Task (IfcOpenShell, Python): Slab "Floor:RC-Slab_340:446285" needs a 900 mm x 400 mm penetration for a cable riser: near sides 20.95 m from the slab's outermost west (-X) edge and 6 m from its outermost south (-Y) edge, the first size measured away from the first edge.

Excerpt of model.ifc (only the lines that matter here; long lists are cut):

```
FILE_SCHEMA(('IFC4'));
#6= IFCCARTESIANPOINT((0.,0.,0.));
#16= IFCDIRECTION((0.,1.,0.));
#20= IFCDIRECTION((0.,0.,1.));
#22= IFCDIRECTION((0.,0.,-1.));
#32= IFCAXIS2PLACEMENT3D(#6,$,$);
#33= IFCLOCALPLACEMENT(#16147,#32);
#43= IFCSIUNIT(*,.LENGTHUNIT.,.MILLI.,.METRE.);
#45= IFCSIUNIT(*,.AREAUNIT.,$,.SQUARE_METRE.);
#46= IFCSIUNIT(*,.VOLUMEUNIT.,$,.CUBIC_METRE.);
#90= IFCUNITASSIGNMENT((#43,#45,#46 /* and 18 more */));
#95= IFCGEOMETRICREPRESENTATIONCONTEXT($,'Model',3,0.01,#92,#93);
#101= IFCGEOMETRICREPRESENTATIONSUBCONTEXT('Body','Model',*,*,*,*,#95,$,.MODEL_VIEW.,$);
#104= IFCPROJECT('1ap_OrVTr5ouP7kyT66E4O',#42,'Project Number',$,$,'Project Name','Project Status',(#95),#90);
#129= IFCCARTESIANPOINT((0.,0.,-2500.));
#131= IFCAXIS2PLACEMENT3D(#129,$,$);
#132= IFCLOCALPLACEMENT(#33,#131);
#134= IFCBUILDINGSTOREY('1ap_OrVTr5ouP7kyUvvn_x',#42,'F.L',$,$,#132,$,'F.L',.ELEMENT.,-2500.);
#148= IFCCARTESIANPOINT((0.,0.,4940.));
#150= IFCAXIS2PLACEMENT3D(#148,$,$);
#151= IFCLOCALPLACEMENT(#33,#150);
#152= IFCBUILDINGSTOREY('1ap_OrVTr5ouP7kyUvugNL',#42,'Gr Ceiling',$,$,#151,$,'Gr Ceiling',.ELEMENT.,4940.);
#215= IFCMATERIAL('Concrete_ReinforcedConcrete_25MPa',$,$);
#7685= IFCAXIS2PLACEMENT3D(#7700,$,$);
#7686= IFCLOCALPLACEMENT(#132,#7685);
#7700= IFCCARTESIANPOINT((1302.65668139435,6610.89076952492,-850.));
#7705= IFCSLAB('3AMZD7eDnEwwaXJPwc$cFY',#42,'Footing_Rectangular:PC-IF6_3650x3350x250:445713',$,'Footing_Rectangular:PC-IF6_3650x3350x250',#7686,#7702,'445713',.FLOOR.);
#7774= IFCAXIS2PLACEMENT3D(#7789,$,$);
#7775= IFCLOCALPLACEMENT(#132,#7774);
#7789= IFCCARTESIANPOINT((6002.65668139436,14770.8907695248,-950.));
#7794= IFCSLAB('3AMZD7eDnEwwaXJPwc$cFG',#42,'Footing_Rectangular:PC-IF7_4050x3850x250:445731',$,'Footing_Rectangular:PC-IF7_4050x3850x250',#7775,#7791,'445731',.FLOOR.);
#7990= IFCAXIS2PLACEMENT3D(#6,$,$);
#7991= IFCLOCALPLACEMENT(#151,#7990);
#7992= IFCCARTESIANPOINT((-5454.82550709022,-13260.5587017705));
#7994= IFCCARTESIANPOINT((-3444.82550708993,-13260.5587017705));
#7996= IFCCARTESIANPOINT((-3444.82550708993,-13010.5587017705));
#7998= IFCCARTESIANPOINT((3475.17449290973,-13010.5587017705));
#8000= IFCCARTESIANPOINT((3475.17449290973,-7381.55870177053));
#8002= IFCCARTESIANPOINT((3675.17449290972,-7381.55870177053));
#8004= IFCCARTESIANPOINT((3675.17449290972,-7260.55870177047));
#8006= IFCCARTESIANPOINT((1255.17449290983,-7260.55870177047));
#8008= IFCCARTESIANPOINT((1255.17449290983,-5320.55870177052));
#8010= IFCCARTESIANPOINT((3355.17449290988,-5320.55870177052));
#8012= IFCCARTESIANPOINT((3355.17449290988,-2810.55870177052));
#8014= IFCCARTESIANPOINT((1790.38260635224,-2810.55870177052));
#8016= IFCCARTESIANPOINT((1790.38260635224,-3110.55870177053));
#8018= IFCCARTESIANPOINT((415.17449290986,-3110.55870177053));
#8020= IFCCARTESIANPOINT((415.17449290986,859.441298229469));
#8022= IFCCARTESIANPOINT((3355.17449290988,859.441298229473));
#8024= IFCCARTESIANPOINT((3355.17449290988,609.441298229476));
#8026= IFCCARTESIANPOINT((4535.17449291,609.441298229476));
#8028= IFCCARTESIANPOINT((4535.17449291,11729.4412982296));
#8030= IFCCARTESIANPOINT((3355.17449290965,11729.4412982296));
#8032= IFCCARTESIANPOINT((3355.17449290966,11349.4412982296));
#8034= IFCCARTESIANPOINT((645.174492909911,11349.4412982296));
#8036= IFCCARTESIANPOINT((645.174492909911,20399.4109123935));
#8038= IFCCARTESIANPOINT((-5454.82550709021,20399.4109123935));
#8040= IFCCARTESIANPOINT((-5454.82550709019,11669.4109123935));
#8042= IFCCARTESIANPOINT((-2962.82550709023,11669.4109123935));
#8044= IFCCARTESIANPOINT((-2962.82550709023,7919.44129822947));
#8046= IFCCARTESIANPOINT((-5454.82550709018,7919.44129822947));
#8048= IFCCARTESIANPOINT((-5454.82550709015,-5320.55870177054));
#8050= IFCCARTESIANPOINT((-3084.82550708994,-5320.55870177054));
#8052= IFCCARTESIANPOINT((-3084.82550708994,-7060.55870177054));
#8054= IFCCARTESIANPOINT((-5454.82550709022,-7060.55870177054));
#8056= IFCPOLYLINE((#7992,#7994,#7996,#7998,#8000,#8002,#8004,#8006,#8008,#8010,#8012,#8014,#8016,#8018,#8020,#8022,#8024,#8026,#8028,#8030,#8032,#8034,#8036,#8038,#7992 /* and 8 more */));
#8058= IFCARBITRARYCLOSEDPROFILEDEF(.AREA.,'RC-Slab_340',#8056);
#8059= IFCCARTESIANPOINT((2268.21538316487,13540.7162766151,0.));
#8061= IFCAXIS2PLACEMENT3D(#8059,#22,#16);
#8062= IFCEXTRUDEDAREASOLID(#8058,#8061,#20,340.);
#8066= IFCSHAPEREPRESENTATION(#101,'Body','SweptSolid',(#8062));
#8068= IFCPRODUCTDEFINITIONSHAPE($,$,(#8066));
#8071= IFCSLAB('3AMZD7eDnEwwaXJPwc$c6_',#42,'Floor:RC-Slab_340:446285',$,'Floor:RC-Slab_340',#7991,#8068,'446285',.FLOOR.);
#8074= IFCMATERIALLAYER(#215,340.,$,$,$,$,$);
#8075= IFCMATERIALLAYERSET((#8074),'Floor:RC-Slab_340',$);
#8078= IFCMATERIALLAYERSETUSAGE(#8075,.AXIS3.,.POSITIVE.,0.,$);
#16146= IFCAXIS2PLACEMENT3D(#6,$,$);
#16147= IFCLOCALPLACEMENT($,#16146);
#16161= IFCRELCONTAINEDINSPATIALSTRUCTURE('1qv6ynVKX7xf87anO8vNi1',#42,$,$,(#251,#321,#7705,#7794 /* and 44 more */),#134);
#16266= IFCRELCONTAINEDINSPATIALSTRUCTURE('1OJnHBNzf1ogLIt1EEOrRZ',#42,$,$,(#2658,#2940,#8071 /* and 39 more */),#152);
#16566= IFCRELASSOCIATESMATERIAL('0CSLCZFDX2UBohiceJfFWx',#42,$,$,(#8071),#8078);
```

```python
import numpy as np
import ifcopenshell
import ifcopenshell.api.feature
import ifcopenshell.api.geometry
import ifcopenshell.api.root
import ifcopenshell.geom
import ifcopenshell.util.placement
import ifcopenshell.util.representation
import ifcopenshell.util.shape
import ifcopenshell.util.unit

model = ifcopenshell.open("model.ifc")
unit_scale = ifcopenshell.util.unit.calculate_unit_scale(model)
settings = ifcopenshell.geom.settings()


def volume(element):
    """Net volume in cubic metres, openings subtracted."""
    shape = ifcopenshell.geom.create_shape(settings, element)
    return ifcopenshell.util.shape.get_volume(shape.geometry)


slab = model.by_guid("3AMZD7eDnEwwaXJPwc$c6_")
before = volume(slab)

# Extent in the slab's own axes, in metres. The edges named are its -X and -Y sides.
slab_shape = ifcopenshell.geom.create_shape(settings, slab)
vertices = ifcopenshell.util.shape.get_vertices(slab_shape.geometry)
x_min, y_min, bottom = vertices.min(axis=0)
top = vertices[:, 2].max()

opening = ifcopenshell.api.root.create_entity(model, ifc_class="IfcOpeningElement", name="Cable riser opening", predefined_type="OPENING")
context = ifcopenshell.util.representation.get_context(model, "Model", "Body", "MODEL_VIEW")
width, depth = 0.9, 0.4
outline = [(0.0, 0.0), (width, 0.0), (width, depth), (0.0, depth), (0.0, 0.0)]
# Overshoot both faces by 50 mm so the cut is clean.
shape = ifcopenshell.api.geometry.add_slab_representation(
    model, context=context, depth=top - bottom + 0.1, polyline=outline
)
ifcopenshell.api.geometry.assign_representation(model, product=opening, representation=shape)

matrix = ifcopenshell.util.placement.get_local_placement(slab.ObjectPlacement)
matrix[:, 3] = matrix @ np.append(np.array([x_min + 20.95, y_min + 6, bottom - 0.05]) / unit_scale, 1.0)
ifcopenshell.api.geometry.edit_object_placement(model, product=opening, matrix=matrix, is_si=False)
ifcopenshell.api.feature.add_feature(model, feature=opening, element=slab)

after = volume(slab)

print(f"slab volume {before:.3f} -> {after:.3f} m3")

model.write("model_edited.ifc")
```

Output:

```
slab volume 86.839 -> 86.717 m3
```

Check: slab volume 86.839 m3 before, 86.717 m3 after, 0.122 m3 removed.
